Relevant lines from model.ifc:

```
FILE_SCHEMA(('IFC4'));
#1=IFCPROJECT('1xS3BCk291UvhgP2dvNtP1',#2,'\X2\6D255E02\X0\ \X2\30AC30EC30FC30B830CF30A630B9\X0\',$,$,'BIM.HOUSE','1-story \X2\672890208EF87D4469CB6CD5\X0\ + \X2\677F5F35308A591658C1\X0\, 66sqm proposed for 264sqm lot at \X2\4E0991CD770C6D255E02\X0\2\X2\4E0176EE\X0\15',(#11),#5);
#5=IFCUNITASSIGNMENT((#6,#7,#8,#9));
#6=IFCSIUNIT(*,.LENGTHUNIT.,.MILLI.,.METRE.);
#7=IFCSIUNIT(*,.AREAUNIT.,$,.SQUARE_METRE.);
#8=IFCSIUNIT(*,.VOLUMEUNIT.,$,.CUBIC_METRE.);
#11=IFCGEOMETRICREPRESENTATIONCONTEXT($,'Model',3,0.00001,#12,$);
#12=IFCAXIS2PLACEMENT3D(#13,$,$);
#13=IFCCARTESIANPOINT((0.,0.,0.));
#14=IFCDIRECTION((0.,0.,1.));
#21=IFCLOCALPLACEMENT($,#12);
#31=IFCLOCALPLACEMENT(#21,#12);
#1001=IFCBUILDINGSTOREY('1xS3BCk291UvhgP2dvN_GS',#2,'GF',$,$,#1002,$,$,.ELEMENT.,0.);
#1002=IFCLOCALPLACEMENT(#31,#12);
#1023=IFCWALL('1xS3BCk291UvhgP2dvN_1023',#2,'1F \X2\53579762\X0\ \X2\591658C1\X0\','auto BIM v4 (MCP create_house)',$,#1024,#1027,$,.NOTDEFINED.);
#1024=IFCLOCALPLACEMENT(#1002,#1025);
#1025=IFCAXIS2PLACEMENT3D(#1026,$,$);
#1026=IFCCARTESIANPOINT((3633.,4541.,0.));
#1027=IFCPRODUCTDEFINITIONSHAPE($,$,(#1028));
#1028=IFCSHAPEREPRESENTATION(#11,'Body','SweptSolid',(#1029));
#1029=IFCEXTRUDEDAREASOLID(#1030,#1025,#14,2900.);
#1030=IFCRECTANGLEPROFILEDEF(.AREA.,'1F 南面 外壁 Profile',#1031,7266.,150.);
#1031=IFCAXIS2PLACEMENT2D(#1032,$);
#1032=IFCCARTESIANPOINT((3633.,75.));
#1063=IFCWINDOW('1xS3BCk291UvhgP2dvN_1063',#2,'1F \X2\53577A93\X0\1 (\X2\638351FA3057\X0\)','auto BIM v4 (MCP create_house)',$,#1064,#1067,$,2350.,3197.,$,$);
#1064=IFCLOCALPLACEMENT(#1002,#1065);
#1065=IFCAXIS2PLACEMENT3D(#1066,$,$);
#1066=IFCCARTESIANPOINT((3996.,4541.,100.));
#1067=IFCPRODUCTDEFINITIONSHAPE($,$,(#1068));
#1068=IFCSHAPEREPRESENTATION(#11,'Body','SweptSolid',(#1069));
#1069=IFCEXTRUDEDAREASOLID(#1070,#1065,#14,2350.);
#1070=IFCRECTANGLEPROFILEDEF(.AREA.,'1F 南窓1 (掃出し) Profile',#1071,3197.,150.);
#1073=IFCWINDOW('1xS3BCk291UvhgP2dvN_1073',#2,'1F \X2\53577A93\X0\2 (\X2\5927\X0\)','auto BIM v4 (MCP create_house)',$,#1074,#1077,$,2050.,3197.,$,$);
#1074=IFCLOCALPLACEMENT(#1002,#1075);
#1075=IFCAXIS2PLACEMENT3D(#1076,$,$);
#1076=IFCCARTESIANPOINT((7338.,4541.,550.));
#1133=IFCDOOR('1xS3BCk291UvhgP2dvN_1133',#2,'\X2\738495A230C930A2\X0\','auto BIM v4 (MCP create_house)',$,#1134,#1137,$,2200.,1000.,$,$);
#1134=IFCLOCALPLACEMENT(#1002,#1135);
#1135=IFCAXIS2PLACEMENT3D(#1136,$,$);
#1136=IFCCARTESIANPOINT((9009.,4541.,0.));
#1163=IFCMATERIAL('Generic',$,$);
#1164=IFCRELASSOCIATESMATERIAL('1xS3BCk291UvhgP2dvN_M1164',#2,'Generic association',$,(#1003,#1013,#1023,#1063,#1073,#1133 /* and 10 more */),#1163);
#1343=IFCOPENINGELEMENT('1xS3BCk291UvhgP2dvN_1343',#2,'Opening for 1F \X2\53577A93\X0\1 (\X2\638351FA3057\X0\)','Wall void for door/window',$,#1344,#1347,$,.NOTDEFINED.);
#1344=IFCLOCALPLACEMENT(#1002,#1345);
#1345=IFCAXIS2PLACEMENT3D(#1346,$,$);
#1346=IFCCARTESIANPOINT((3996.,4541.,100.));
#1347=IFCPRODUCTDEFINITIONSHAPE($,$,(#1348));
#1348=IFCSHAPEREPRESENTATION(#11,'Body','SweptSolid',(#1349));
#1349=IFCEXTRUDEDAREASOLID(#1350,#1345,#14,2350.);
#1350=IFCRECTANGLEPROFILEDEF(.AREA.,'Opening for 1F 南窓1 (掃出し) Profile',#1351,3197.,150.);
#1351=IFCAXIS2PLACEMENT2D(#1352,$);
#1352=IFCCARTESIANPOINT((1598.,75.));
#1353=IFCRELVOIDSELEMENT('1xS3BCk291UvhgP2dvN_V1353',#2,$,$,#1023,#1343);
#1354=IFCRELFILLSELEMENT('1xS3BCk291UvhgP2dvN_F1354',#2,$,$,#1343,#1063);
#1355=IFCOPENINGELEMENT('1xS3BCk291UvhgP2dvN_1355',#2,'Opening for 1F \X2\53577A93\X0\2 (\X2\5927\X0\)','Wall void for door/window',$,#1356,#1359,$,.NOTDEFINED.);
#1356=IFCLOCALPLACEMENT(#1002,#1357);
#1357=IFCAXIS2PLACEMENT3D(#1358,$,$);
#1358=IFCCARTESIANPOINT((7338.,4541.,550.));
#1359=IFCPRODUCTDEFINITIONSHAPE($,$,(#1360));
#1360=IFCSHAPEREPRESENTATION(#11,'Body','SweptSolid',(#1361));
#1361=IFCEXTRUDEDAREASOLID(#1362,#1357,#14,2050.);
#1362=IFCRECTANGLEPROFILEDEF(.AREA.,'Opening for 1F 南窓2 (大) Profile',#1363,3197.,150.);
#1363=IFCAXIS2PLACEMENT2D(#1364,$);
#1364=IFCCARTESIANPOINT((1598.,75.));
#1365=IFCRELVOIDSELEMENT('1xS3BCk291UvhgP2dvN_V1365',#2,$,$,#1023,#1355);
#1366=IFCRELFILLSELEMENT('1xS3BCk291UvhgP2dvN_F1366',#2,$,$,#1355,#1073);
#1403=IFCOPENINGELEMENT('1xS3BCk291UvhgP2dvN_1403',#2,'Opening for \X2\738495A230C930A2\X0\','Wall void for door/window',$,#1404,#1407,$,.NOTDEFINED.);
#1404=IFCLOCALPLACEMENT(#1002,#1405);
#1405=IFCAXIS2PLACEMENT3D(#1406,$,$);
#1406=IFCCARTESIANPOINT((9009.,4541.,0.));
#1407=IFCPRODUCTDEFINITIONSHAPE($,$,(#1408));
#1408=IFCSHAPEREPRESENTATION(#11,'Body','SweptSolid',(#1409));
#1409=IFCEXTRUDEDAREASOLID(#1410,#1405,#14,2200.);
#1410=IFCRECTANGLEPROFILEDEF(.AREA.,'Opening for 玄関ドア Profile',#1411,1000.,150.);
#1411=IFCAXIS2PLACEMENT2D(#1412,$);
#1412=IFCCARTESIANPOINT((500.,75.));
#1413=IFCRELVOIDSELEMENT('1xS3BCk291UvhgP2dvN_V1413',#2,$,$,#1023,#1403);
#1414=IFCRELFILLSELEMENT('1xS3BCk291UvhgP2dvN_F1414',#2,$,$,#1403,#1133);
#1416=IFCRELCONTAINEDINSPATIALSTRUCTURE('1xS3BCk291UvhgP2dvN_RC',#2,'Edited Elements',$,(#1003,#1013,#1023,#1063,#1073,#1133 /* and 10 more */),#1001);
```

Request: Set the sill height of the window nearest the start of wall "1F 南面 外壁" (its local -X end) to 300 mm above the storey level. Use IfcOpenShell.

```python
import numpy as np
import ifcopenshell
import ifcopenshell.api.geometry
import ifcopenshell.geom
import ifcopenshell.util.element
import ifcopenshell.util.placement
import ifcopenshell.util.shape
import ifcopenshell.util.unit

model = ifcopenshell.open("model.ifc")
unit_scale = ifcopenshell.util.unit.calculate_unit_scale(model)

window = model.by_guid("1xS3BCk291UvhgP2dvN_1063")
opening = window.FillsVoids[0].RelatingOpeningElement
storey = ifcopenshell.util.element.get_container(window, ifc_class="IfcBuildingStorey")
level = ifcopenshell.util.placement.get_local_placement(storey.ObjectPlacement)[2, 3]

# The opening's origin need not be at the sill, so measure its lowest point.
shape = ifcopenshell.geom.create_shape(ifcopenshell.geom.settings(), opening)
bottom = ifcopenshell.util.shape.get_shape_bottom_elevation(shape, shape.geometry) / unit_scale
dz = level + 0.3 / unit_scale - bottom

shift = np.array([0.0, 0.0, dz])
# The window is not placed relative to its opening, so move both.
for product in (opening, window):
    matrix = ifcopenshell.util.placement.get_local_placement(product.ObjectPlacement)
    matrix[:3, 3] += shift
    ifcopenshell.api.geometry.edit_object_placement(model, product=product, matrix=matrix, is_si=False)

print(f"moved by {dz * unit_scale:+.3f} m")

model.write("model-out.ifc")
```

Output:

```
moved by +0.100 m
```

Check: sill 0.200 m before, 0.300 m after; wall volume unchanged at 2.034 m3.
